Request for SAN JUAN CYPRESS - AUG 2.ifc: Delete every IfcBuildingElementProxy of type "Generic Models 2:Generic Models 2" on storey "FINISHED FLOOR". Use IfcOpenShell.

First a look at what the model holds.

```python
import ifcopenshell
import ifcopenshell.util.element

model = ifcopenshell.open("SAN JUAN CYPRESS - AUG 2.ifc")
print(model.schema)
storey = next(s for s in model.by_type("IfcBuildingStorey") if s.Name == "FINISHED FLOOR")
proxies = [e for e in ifcopenshell.util.element.get_decomposition(storey) if e.is_a("IfcBuildingElementProxy")]
seen = {}
for e in proxies:
    element_type = ifcopenshell.util.element.get_type(e)
    name = element_type.Name if element_type not in (None, e) else None
    seen[name] = seen.get(name, 0) + 1
for name, count in sorted(seen.items(), key=str):
    print(count, "x", name)
```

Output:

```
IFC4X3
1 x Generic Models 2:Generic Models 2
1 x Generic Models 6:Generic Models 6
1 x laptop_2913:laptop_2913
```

```python
import ifcopenshell
import ifcopenshell.api.root
import ifcopenshell.util.element

model = ifcopenshell.open("SAN JUAN CYPRESS - AUG 2.ifc")

storey = next(s for s in model.by_type("IfcBuildingStorey") if s.Name == "FINISHED FLOOR")
proxies = [e for e in ifcopenshell.util.element.get_decomposition(storey) if e.is_a("IfcBuildingElementProxy")]
targets = [e for e in proxies if (t := ifcopenshell.util.element.get_type(e)) not in (None, e) and t.Name == "Generic Models 2:Generic Models 2"]

for e in targets:
    ifcopenshell.api.root.remove_product(model, product=e)
print(len(targets), "removed")

model.write("SAN JUAN CYPRESS - AUG 2_v2.ifc")
```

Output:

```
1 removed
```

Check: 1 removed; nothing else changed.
